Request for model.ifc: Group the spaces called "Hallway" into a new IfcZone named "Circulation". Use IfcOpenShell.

First a look at what the model holds.

```python
import ifcopenshell

model = ifcopenshell.open("model.ifc")
print(model.schema)
seen = {}
for space in model.by_type("IfcSpace"):
    seen[space.LongName] = seen.get(space.LongName, 0) + 1
for name, count in sorted(seen.items(), key=str):
    print(count, "x", name)
print("zones:", [z.Name for z in model.by_type("IfcZone")][:20])
```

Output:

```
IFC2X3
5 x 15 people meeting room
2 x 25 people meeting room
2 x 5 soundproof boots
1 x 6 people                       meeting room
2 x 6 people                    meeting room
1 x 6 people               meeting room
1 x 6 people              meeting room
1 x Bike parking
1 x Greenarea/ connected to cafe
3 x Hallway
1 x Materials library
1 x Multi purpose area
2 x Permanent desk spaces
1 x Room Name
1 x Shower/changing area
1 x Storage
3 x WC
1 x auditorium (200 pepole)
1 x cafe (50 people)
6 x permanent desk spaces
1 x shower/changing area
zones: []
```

```python
import ifcopenshell
import ifcopenshell.api.group
import ifcopenshell.api.root

model = ifcopenshell.open("model.ifc")

names = {"Hallway"}
spaces = [s for s in model.by_type("IfcSpace") if s.LongName in names]

zone = ifcopenshell.api.root.create_entity(model, ifc_class="IfcZone", name="Circulation")
ifcopenshell.api.group.assign_group(model, products=spaces, group=zone)
print(len(spaces), "spaces in", zone.Name)

model.write("model_v2.ifc")
```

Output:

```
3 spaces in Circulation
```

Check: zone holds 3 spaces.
